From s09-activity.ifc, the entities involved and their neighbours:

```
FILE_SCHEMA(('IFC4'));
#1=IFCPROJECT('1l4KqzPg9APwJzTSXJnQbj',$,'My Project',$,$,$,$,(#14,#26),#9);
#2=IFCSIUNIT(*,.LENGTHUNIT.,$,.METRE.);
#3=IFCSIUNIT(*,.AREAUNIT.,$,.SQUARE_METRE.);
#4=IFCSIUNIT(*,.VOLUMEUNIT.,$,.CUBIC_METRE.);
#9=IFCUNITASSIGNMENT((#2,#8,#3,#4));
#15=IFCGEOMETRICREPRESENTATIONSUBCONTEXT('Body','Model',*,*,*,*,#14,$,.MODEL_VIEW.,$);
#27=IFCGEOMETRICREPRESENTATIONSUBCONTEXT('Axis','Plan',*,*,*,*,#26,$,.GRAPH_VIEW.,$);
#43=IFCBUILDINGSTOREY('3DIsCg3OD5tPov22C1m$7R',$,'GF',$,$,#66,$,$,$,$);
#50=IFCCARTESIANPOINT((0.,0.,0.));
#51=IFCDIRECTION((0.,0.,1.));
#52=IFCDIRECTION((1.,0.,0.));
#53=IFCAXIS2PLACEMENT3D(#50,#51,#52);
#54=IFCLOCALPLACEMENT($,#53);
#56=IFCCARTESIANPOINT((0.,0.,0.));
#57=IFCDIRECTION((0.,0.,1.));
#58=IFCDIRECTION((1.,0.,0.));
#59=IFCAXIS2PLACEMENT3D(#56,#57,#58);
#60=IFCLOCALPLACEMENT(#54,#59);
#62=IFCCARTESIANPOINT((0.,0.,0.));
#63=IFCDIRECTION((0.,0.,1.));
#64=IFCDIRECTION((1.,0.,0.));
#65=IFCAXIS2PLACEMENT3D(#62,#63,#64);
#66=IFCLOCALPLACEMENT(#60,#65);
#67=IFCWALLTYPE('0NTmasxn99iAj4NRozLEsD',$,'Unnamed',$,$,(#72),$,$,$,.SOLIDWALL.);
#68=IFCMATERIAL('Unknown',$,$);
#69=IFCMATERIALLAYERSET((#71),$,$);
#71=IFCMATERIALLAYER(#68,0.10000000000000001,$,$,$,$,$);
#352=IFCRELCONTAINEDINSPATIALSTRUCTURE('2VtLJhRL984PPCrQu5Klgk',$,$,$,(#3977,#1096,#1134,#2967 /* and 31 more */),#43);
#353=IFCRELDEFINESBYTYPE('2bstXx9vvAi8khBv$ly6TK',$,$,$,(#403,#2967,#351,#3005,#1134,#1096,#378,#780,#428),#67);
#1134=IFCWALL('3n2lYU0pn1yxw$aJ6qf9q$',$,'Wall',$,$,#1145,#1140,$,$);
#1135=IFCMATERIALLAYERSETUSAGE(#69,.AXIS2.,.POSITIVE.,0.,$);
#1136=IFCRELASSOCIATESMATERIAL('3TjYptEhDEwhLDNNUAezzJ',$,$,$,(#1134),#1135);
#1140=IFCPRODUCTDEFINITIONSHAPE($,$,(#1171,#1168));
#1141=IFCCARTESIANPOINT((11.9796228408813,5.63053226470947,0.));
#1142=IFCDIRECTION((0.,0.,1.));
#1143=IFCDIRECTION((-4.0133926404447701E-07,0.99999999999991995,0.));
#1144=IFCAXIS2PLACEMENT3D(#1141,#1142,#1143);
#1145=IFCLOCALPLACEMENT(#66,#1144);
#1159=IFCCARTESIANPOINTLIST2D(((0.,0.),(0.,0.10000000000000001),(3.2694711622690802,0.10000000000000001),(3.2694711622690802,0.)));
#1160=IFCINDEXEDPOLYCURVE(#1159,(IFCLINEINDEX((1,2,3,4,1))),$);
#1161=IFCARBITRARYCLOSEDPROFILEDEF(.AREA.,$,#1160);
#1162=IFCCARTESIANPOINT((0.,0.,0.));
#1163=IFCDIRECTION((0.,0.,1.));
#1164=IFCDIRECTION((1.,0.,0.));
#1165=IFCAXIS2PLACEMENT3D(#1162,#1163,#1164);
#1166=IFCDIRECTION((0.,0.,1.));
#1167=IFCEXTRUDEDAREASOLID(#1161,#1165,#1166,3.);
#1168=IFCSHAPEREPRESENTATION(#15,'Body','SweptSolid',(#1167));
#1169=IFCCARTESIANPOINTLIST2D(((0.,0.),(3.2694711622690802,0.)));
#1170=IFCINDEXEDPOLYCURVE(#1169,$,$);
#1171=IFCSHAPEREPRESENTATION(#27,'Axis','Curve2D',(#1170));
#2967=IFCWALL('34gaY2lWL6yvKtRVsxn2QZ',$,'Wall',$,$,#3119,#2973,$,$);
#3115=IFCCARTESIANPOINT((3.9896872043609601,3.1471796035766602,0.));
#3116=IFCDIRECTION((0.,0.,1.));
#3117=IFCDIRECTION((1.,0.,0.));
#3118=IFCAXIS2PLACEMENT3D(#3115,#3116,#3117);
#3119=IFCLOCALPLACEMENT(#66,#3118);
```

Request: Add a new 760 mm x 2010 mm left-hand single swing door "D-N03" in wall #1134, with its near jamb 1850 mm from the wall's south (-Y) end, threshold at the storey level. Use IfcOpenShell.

```python
import numpy as np
import ifcopenshell
import ifcopenshell.api.feature
import ifcopenshell.api.geometry
import ifcopenshell.api.root
import ifcopenshell.api.spatial
import ifcopenshell.geom
import ifcopenshell.util.element
import ifcopenshell.util.placement
import ifcopenshell.util.representation
import ifcopenshell.util.shape
import ifcopenshell.util.unit

model = ifcopenshell.open("s09-activity.ifc")
unit_scale = ifcopenshell.util.unit.calculate_unit_scale(model)
settings = ifcopenshell.geom.settings()


def volume(element):
    """Net volume in cubic metres, openings subtracted."""
    shape = ifcopenshell.geom.create_shape(settings, element)
    return ifcopenshell.util.shape.get_volume(shape.geometry)


wall = model.by_guid("3n2lYU0pn1yxw$aJ6qf9q$")
storey = ifcopenshell.util.element.get_container(wall, ifc_class="IfcBuildingStorey")
context = ifcopenshell.util.representation.get_context(model, "Model", "Body", "MODEL_VIEW")
before = volume(wall)

width, height, from_end, sill = 0.76, 2.01, 1.85, 0.0  # metres

# The wall runs along its own X axis, and the end named is its -X end.
wall_shape = ifcopenshell.geom.create_shape(settings, wall)
x, y, z = ifcopenshell.util.shape.get_vertices(wall_shape.geometry).T
start = x.min() + from_end
face, thickness = float(y.min()), float(y.max() - y.min())
wall_matrix = ifcopenshell.util.placement.get_local_placement(wall.ObjectPlacement)
level = ifcopenshell.util.placement.get_local_placement(storey.ObjectPlacement)[2, 3]


def in_wall(x, y):
    """Placement at x, y metres in the wall's axes, at sill height."""
    matrix = wall_matrix.copy()
    matrix[:, 3] = wall_matrix @ np.array([x / unit_scale, y / unit_scale, 0.0, 1.0])
    matrix[2, 3] = level + sill / unit_scale
    return matrix


# Opening: a box that overshoots both wall faces by 50 mm.
opening = ifcopenshell.api.root.create_entity(model, ifc_class="IfcOpeningElement", predefined_type="OPENING")
box = ifcopenshell.api.geometry.add_wall_representation(
    model, context=context, length=width, height=height, thickness=thickness + 0.1
)
ifcopenshell.api.geometry.assign_representation(model, product=opening, representation=box)
ifcopenshell.api.geometry.edit_object_placement(model, product=opening, matrix=in_wall(start, face - 0.05), is_si=False)
ifcopenshell.api.feature.add_feature(model, feature=opening, element=wall)

door = ifcopenshell.api.root.create_entity(model, ifc_class="IfcDoor", name="D-N03", predefined_type="DOOR")
door.OverallWidth, door.OverallHeight = width / unit_scale, height / unit_scale
door.OperationType = "SINGLE_SWING_LEFT"
body = ifcopenshell.api.geometry.add_door_representation(
    model,
    context=context,
    overall_width=door.OverallWidth,
    overall_height=door.OverallHeight,
    operation_type="SINGLE_SWING_LEFT",
    lining_properties={"LiningDepth": thickness / unit_scale, "ThresholdDepth": thickness / unit_scale},
)
ifcopenshell.api.geometry.assign_representation(model, product=door, representation=body)
ifcopenshell.api.spatial.assign_container(model, products=[door], relating_structure=storey)
ifcopenshell.api.feature.add_filling(model, opening=opening, element=door)

# The lining spans the wall, so the door starts at the wall face.
ifcopenshell.api.geometry.edit_object_placement(model, product=door, matrix=in_wall(start, face), is_si=False)

after = volume(wall)

print(f"wall volume {before:.3f} -> {after:.3f} m3")

model.write("s09-activity_updated.ifc")
```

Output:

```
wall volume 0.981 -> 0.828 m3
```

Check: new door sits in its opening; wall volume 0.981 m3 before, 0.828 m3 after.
